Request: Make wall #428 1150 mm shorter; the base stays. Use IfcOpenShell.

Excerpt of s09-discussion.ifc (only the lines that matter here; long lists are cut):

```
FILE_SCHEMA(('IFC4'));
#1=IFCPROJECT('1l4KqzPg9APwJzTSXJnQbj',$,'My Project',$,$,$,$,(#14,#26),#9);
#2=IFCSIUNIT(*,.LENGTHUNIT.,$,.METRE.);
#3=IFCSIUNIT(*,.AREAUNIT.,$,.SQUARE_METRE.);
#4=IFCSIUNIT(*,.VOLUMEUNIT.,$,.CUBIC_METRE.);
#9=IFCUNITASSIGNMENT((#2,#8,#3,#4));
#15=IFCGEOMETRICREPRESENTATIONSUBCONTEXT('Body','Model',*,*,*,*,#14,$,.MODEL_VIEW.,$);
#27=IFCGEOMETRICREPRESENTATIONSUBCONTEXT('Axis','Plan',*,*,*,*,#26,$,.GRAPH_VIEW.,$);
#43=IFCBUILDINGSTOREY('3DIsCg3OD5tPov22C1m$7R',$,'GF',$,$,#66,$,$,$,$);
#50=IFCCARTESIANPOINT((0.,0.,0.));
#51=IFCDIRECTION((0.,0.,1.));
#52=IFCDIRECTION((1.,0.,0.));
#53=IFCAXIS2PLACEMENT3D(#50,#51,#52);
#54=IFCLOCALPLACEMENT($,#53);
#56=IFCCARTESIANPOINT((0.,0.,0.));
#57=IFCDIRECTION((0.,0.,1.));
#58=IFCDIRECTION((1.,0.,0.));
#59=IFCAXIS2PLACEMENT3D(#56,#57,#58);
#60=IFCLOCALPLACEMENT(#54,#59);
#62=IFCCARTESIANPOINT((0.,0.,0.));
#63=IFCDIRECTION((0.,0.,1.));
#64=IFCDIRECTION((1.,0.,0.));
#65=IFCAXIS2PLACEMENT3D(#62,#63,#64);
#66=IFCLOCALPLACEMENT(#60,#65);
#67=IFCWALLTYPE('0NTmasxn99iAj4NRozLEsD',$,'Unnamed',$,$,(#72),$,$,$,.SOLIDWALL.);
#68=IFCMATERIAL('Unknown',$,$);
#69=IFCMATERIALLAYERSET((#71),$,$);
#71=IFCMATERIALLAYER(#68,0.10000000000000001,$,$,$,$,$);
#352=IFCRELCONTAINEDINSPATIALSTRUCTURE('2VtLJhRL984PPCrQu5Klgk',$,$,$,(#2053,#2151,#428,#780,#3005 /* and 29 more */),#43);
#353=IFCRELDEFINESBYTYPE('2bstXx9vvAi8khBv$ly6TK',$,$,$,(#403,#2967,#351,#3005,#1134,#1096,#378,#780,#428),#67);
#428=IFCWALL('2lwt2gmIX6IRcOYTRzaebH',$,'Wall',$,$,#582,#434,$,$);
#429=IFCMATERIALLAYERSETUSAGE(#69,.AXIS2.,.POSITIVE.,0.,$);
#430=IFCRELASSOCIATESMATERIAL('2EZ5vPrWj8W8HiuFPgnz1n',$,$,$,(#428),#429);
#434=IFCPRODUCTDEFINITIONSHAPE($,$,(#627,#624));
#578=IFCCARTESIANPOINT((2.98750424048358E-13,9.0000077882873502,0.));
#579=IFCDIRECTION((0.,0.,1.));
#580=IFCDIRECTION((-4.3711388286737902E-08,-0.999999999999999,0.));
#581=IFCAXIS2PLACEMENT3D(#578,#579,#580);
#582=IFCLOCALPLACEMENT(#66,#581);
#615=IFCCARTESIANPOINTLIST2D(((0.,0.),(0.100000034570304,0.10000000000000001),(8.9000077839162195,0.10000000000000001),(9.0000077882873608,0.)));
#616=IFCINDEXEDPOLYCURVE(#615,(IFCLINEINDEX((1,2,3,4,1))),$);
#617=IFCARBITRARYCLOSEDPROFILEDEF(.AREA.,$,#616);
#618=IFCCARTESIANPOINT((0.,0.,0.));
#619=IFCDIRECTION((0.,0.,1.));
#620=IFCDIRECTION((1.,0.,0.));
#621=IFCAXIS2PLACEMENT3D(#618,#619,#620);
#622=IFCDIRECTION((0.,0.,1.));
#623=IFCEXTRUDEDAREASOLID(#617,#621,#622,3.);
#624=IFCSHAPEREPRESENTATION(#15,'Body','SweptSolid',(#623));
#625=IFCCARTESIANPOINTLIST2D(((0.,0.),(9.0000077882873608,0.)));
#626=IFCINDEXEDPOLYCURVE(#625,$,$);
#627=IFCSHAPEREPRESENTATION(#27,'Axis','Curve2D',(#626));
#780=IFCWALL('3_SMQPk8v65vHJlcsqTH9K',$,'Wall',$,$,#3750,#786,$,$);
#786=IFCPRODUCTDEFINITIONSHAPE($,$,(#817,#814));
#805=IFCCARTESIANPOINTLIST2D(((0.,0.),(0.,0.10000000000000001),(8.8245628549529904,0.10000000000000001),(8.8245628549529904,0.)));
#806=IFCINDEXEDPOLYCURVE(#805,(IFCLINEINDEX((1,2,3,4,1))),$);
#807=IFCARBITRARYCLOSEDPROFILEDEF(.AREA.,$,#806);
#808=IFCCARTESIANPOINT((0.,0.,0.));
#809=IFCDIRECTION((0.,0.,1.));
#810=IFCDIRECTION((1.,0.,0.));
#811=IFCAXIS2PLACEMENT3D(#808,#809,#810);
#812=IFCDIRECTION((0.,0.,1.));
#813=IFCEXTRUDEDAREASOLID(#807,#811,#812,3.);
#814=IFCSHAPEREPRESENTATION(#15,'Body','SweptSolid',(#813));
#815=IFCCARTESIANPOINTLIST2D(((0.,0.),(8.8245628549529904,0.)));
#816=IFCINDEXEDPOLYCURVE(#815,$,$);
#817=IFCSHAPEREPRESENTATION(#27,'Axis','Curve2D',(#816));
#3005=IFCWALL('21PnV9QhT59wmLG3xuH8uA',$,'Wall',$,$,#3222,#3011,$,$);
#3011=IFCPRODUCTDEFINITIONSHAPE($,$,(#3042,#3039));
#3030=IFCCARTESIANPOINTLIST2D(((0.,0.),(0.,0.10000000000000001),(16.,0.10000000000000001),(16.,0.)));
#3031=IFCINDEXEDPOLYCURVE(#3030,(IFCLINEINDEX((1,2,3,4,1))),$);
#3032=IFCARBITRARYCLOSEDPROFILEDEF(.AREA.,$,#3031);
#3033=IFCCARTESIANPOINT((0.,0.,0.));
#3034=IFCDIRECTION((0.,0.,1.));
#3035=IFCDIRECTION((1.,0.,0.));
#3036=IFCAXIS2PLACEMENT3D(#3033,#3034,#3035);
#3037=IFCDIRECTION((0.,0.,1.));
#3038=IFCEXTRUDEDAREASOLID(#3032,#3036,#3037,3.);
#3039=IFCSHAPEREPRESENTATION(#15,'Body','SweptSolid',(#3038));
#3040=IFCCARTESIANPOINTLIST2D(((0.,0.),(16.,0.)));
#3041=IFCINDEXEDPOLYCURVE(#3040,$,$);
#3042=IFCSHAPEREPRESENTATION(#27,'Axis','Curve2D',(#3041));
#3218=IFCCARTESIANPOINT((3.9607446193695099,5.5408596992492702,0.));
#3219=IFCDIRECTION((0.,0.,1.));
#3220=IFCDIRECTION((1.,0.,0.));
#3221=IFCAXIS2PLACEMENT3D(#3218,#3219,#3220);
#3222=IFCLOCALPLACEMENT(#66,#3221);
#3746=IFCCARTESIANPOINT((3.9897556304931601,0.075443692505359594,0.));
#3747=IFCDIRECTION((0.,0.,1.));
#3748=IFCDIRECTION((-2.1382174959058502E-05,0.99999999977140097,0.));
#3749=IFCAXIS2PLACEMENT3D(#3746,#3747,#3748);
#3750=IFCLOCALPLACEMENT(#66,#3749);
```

```python
import ifcopenshell
import ifcopenshell.geom
import ifcopenshell.util.representation
import ifcopenshell.util.shape
import ifcopenshell.util.unit

model = ifcopenshell.open("s09-discussion.ifc")
unit_scale = ifcopenshell.util.unit.calculate_unit_scale(model)
settings = ifcopenshell.geom.settings()


def volume(element):
    """Net volume in cubic metres, openings subtracted."""
    shape = ifcopenshell.geom.create_shape(settings, element)
    return ifcopenshell.util.shape.get_volume(shape.geometry)


wall = model.by_guid("2lwt2gmIX6IRcOYTRzaebH")
before = volume(wall)

body = ifcopenshell.util.representation.get_representation(wall, "Model", "Body")
solid = body.Items[0]
old_height = solid.Depth
solid.Depth -= 1.15 / unit_scale
after = volume(wall)

print(f"height {old_height:g} -> {solid.Depth:g}, volume {before:.3f} -> {after:.3f} m3")

model.write("s09-discussion-out.ifc")
```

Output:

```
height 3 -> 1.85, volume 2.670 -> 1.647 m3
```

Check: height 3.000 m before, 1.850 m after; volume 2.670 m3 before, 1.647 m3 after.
